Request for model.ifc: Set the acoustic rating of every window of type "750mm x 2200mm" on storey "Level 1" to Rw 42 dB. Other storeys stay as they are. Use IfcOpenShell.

First a look at what the model holds.

```python
import ifcopenshell
import ifcopenshell.util.element

model = ifcopenshell.open("model.ifc")
print(model.schema)
storey = next(s for s in model.by_type("IfcBuildingStorey") if s.Name == "Level 1")
windows = [e for e in ifcopenshell.util.element.get_decomposition(storey) if e.is_a("IfcWindow")]
seen = {}
for e in windows:
    element_type = ifcopenshell.util.element.get_type(e)
    key = (element_type.Name if element_type != e and element_type else None, ifcopenshell.util.element.get_pset(e, "Pset_WindowCommon", "AcousticRating"))
    seen[key] = seen.get(key, 0) + 1
for (name, value), count in sorted(seen.items(), key=str):
    print(count, "x", name, "|", value)
```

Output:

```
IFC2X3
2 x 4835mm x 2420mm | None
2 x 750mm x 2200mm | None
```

```python
import ifcopenshell
import ifcopenshell.api.pset
import ifcopenshell.util.element

model = ifcopenshell.open("model.ifc")

storey = next(s for s in model.by_type("IfcBuildingStorey") if s.Name == "Level 1")
windows = [e for e in ifcopenshell.util.element.get_decomposition(storey) if e.is_a("IfcWindow")]

count = 0
for e in windows:
    element_type = ifcopenshell.util.element.get_type(e)
    if element_type in (None, e) or element_type.Name != "750mm x 2200mm":
        continue
    # add_pset returns the element's existing set when there is one.
    pset = ifcopenshell.api.pset.add_pset(model, product=e, name="Pset_WindowCommon")
    ifcopenshell.api.pset.edit_pset(model, pset=pset, properties={"AcousticRating": "Rw 42 dB"})
    count += 1

print(count, "windows updated")

model.write("model_edited.ifc")
```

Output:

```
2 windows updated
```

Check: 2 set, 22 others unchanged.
